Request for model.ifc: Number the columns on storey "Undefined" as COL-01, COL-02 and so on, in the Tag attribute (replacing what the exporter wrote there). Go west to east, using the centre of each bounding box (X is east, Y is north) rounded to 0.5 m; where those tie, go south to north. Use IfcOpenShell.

First a look at what the model holds.

```python
import ifcopenshell
import ifcopenshell.util.element
import ifcopenshell.util.placement

model = ifcopenshell.open("model.ifc")
print(model.schema)
storey = next(s for s in model.by_type("IfcBuildingStorey") if s.Name == "Undefined")
columns = [e for e in ifcopenshell.util.element.get_decomposition(storey) if e.is_a("IfcColumn")]
for e in sorted(columns, key=lambda e: e.id()):
    origin = ifcopenshell.util.placement.get_local_placement(e.ObjectPlacement)[:3, 3]
    print(e.id(), e.Tag, e.Name, origin.round(2) + 0.0, sep=" | ")
```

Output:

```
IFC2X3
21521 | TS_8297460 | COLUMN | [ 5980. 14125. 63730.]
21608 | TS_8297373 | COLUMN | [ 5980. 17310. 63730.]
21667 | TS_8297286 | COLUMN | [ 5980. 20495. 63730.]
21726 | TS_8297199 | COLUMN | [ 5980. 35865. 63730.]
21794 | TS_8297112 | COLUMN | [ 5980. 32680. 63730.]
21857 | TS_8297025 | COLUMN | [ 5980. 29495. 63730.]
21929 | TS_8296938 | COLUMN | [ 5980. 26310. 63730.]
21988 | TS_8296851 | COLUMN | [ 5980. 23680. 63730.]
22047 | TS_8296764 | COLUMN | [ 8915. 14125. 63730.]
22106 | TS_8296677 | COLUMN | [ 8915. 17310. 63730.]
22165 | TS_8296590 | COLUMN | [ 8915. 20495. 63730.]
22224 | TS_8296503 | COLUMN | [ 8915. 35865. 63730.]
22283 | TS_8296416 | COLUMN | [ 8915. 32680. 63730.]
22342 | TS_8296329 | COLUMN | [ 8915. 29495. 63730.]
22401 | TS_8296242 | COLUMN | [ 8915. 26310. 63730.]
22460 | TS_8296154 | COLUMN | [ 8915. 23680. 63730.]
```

```python
import ifcopenshell
import ifcopenshell.geom
import ifcopenshell.util.element
import ifcopenshell.util.shape

model = ifcopenshell.open("model.ifc")
settings = ifcopenshell.geom.settings()
settings.set("use-world-coords", True)


def centre(element):
    shape = ifcopenshell.geom.create_shape(settings, element)
    return ifcopenshell.util.shape.get_bbox_centroid(shape.geometry)


storey = next(s for s in model.by_type("IfcBuildingStorey") if s.Name == "Undefined")
columns = [e for e in ifcopenshell.util.element.get_decomposition(storey) if e.is_a("IfcColumn")]

# Insertion points can sit at a corner or the storey origin, so sort by the geometry (in metres).
centres = {e: centre(e) for e in columns}
columns.sort(key=lambda e: (round(centres[e][0] / 0.5), centres[e][1]))

for i, e in enumerate(columns, start=1):
    number = f"COL-{i:02d}"
    e.Tag = number
    print(e.id(), number)

model.write("model_v2.ifc")
```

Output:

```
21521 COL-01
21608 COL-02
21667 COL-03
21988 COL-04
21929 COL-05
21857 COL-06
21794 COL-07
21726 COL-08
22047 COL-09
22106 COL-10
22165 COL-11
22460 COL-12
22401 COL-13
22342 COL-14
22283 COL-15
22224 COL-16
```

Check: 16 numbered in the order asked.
